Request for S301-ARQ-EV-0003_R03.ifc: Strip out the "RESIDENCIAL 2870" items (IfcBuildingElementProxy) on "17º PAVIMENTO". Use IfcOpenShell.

First a look at what the model holds.

```python
import ifcopenshell
import ifcopenshell.util.element

model = ifcopenshell.open("S301-ARQ-EV-0003_R03.ifc")
print(model.schema)
storey = next(s for s in model.by_type("IfcBuildingStorey") if s.Name == "17º PAVIMENTO")
proxies = [e for e in ifcopenshell.util.element.get_decomposition(storey) if e.is_a("IfcBuildingElementProxy")]
seen = {}
for e in proxies:
    element_type = ifcopenshell.util.element.get_type(e)
    name = element_type.Name if element_type not in (None, e) else None
    seen[name] = seen.get(name, 0) + 1
for name, count in sorted(seen.items(), key=str):
    print(count, "x", name)
```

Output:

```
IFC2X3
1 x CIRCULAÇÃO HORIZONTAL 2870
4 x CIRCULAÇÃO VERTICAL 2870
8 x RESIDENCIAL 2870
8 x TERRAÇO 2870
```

```python
import ifcopenshell
import ifcopenshell.api.root
import ifcopenshell.util.element

model = ifcopenshell.open("S301-ARQ-EV-0003_R03.ifc")

storey = next(s for s in model.by_type("IfcBuildingStorey") if s.Name == "17º PAVIMENTO")
proxies = [e for e in ifcopenshell.util.element.get_decomposition(storey) if e.is_a("IfcBuildingElementProxy")]
targets = [e for e in proxies if (t := ifcopenshell.util.element.get_type(e)) not in (None, e) and t.Name == "RESIDENCIAL 2870"]

for e in targets:
    ifcopenshell.api.root.remove_product(model, product=e)
print(len(targets), "removed")

model.write("S301-ARQ-EV-0003_R03_rev.ifc")
```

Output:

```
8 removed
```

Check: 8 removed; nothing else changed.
